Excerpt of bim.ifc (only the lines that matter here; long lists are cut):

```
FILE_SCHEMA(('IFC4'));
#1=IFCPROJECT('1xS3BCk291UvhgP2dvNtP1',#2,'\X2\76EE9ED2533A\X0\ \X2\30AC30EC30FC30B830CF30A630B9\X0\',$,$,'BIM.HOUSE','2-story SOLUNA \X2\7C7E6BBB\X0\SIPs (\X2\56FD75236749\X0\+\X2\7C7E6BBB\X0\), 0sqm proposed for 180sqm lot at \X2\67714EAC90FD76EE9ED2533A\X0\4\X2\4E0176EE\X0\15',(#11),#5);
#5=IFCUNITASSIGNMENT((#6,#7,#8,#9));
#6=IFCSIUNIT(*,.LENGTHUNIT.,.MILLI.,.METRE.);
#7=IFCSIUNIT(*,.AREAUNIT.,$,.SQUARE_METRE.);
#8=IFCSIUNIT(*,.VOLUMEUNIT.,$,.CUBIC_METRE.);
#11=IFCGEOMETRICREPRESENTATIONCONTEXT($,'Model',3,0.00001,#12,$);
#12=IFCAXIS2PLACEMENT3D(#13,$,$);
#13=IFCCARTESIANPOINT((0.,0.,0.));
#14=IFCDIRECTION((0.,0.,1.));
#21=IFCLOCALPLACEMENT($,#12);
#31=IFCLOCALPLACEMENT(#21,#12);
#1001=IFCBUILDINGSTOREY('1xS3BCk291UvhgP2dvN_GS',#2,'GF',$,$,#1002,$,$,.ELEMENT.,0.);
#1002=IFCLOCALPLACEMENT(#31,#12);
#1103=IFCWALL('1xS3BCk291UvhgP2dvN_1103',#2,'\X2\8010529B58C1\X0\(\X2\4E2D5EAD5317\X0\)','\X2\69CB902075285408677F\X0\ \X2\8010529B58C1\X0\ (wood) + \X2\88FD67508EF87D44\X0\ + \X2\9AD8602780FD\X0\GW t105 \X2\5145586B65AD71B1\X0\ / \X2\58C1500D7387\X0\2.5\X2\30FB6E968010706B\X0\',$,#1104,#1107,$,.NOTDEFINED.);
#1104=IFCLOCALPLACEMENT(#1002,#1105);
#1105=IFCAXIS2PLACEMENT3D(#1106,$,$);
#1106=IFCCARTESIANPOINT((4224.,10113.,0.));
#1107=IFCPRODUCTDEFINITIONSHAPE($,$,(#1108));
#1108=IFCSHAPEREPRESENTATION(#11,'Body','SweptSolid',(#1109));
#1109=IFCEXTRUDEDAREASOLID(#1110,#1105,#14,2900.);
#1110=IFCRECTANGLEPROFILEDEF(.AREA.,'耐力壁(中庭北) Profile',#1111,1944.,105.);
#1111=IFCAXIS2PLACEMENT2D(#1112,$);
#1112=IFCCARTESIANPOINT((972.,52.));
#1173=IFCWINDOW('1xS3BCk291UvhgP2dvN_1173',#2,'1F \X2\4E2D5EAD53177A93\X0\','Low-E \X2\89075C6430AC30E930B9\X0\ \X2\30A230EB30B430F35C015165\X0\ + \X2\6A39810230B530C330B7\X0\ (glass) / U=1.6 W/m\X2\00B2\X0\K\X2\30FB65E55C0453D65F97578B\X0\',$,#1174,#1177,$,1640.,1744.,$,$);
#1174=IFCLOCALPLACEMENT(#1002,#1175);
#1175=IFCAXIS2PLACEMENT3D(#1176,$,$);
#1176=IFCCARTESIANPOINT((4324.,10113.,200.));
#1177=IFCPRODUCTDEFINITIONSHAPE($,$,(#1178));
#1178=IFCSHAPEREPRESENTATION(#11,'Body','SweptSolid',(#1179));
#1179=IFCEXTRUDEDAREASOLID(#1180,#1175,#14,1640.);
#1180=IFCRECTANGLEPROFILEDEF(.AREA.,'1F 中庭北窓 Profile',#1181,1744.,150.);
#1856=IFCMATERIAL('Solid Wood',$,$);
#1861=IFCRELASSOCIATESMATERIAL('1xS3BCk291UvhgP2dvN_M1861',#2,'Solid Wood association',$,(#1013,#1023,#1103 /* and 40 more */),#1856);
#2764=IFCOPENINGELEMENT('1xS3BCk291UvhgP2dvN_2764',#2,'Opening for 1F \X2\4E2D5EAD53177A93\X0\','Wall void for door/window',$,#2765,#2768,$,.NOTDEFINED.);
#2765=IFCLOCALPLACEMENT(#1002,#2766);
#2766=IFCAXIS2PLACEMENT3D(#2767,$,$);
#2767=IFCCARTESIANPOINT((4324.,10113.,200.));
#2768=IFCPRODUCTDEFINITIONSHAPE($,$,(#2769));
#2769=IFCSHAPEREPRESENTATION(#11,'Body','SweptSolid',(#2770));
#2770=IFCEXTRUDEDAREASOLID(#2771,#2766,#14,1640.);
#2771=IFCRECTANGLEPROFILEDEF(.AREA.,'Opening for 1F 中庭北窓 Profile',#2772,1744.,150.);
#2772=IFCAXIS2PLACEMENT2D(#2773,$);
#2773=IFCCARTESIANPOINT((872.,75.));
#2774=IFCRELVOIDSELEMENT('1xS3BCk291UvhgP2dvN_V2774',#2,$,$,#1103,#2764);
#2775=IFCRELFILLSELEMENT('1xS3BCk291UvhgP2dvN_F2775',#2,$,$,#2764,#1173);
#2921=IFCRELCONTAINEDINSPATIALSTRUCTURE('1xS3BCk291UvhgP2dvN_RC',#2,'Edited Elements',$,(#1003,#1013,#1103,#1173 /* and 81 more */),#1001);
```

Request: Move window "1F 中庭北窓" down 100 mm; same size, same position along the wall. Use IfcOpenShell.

```python
import numpy as np
import ifcopenshell
import ifcopenshell.api.geometry
import ifcopenshell.util.placement
import ifcopenshell.util.unit

model = ifcopenshell.open("bim.ifc")
unit_scale = ifcopenshell.util.unit.calculate_unit_scale(model)

window = model.by_guid("1xS3BCk291UvhgP2dvN_1173")
opening = window.FillsVoids[0].RelatingOpeningElement
dz = -100.0

shift = np.array([0.0, 0.0, dz])
# The window is not placed relative to its opening, so move both.
for product in (opening, window):
    matrix = ifcopenshell.util.placement.get_local_placement(product.ObjectPlacement)
    matrix[:3, 3] += shift
    ifcopenshell.api.geometry.edit_object_placement(model, product=product, matrix=matrix, is_si=False)

print(f"moved by {dz * unit_scale:+.3f} m")

model.write("bim-out.ifc")
```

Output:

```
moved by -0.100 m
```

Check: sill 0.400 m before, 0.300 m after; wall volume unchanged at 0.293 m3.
